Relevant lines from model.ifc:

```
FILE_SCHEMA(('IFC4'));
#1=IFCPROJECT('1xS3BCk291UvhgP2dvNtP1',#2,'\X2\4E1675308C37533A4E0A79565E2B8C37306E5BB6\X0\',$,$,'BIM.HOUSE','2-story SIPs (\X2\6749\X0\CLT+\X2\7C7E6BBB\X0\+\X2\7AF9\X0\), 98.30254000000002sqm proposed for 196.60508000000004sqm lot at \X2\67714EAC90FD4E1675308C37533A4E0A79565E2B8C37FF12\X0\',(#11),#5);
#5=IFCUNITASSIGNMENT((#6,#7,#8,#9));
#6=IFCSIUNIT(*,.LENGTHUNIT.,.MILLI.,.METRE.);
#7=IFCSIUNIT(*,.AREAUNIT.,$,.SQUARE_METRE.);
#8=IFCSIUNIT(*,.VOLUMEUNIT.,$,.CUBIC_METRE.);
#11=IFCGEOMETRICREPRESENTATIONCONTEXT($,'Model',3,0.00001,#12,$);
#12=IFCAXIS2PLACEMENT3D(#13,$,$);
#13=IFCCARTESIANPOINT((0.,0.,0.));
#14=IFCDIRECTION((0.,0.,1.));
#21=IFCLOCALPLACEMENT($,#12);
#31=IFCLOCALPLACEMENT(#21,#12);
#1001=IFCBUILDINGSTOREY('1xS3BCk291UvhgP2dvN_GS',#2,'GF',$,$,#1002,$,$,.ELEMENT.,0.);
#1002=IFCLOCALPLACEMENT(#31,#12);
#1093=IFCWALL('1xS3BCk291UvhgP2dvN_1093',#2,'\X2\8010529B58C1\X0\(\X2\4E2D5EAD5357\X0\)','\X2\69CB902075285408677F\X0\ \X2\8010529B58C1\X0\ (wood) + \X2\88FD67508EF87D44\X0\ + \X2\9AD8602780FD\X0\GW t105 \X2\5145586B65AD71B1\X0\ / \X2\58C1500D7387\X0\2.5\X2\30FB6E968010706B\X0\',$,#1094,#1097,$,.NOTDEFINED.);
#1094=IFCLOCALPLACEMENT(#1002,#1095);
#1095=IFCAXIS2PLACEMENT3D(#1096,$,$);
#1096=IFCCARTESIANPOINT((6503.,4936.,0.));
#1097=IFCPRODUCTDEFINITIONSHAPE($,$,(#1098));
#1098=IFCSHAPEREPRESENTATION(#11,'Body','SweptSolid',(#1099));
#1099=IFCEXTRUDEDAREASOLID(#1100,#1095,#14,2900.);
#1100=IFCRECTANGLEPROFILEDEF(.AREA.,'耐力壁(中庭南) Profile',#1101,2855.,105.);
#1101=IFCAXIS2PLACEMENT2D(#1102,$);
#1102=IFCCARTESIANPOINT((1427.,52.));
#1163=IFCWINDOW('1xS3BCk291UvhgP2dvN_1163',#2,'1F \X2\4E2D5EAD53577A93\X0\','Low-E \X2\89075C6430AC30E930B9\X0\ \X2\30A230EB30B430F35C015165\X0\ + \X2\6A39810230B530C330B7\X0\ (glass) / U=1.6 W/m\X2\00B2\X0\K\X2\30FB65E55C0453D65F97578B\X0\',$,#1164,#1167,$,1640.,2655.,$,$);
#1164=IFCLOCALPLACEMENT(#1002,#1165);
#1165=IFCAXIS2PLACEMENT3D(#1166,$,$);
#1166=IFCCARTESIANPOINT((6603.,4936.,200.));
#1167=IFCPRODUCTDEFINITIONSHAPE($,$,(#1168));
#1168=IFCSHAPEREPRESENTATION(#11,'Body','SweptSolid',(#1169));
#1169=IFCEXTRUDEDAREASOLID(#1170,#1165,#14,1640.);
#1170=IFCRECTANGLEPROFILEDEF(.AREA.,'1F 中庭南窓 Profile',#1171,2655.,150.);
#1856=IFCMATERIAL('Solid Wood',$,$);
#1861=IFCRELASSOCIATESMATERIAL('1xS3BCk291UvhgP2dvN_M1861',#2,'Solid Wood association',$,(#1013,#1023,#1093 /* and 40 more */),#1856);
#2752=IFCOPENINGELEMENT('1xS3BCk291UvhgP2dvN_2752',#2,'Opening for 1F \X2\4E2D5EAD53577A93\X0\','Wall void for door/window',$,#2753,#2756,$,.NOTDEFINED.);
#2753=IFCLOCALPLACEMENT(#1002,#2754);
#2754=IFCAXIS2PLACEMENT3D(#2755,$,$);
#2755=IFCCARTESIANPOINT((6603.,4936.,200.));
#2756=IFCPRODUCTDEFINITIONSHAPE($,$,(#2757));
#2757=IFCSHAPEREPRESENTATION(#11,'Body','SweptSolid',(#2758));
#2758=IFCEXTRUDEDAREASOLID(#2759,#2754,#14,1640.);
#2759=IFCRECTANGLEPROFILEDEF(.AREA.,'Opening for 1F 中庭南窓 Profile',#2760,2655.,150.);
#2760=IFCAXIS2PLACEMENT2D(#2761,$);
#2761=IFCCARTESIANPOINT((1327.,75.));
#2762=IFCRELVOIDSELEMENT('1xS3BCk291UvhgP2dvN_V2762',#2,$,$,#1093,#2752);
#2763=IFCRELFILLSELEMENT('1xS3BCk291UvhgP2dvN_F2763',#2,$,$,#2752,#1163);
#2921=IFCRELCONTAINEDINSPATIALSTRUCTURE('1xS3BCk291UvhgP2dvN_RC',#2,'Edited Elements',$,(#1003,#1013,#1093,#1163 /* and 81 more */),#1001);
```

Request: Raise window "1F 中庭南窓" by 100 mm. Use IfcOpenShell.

```python
import numpy as np
import ifcopenshell
import ifcopenshell.api.geometry
import ifcopenshell.util.placement
import ifcopenshell.util.unit

model = ifcopenshell.open("model.ifc")
unit_scale = ifcopenshell.util.unit.calculate_unit_scale(model)

window = model.by_guid("1xS3BCk291UvhgP2dvN_1163")
opening = window.FillsVoids[0].RelatingOpeningElement
dz = 100.0

shift = np.array([0.0, 0.0, dz])
# The window is not placed relative to its opening, so move both.
for product in (opening, window):
    matrix = ifcopenshell.util.placement.get_local_placement(product.ObjectPlacement)
    matrix[:3, 3] += shift
    ifcopenshell.api.geometry.edit_object_placement(model, product=product, matrix=matrix, is_si=False)

print(f"moved by {dz * unit_scale:+.3f} m")

model.write("model_updated.ifc")
```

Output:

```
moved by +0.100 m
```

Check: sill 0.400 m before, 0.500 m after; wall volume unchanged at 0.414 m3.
